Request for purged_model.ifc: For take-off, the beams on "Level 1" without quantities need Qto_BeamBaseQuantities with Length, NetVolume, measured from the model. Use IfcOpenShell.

First a look at what the model holds.

```python
import ifcopenshell
import ifcopenshell.util.element
import ifcopenshell.util.unit

model = ifcopenshell.open("purged_model.ifc")
print(model.schema)
for unit_type in ("LENGTHUNIT", "AREAUNIT", "VOLUMEUNIT"):
    print(unit_type, ifcopenshell.util.unit.calculate_unit_scale(model, unit_type))
storey = next(s for s in model.by_type("IfcBuildingStorey") if s.Name == "Level 1")
beams = [e for e in ifcopenshell.util.element.get_decomposition(storey) if e.is_a("IfcBeam")]
for e in sorted(beams, key=lambda e: e.id()):
    print(e.id(), e.is_a(), e.Name, list(ifcopenshell.util.element.get_psets(e, qtos_only=True)), sep=" | ")
```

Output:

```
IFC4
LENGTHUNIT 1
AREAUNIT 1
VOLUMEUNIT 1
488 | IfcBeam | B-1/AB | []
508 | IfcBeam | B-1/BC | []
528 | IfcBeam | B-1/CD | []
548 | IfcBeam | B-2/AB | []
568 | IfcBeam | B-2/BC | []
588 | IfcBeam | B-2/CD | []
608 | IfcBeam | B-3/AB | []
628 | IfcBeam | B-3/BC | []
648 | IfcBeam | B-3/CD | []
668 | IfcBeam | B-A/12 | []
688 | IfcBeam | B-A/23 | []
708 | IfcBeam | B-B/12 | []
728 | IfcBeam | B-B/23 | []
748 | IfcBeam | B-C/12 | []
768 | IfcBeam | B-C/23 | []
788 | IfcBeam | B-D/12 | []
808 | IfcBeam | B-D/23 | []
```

```python
import ifcopenshell
import ifcopenshell.api.pset
import ifcopenshell.geom
import ifcopenshell.util.element
import ifcopenshell.util.shape
import ifcopenshell.util.unit

model = ifcopenshell.open("purged_model.ifc")
unit_scale = ifcopenshell.util.unit.calculate_unit_scale(model)
volume_scale = ifcopenshell.util.unit.calculate_unit_scale(model, "VOLUMEUNIT")
settings = ifcopenshell.geom.settings()

storey = next(s for s in model.by_type("IfcBuildingStorey") if s.Name == "Level 1")
beams = [e for e in ifcopenshell.util.element.get_decomposition(storey) if e.is_a("IfcBeam")]

for e in sorted(beams, key=lambda e: e.id()):
    if ifcopenshell.util.element.get_psets(e, qtos_only=True, should_inherit=False):
        continue
    # Geometry comes back in metres, in the element's own axes.
    shape = ifcopenshell.geom.create_shape(settings, e)
    values = {
        "Length": ifcopenshell.util.shape.get_max_xyz(shape.geometry) / unit_scale,
        "NetVolume": ifcopenshell.util.shape.get_volume(shape.geometry) / volume_scale,
    }
    qto = ifcopenshell.api.pset.add_qto(model, product=e, name="Qto_BeamBaseQuantities")
    ifcopenshell.api.pset.edit_qto(model, qto=qto, properties=values)
    print(e.id(), {k: round(v, 3) for k, v in values.items()})

model.write("purged_model_rev.ifc")
```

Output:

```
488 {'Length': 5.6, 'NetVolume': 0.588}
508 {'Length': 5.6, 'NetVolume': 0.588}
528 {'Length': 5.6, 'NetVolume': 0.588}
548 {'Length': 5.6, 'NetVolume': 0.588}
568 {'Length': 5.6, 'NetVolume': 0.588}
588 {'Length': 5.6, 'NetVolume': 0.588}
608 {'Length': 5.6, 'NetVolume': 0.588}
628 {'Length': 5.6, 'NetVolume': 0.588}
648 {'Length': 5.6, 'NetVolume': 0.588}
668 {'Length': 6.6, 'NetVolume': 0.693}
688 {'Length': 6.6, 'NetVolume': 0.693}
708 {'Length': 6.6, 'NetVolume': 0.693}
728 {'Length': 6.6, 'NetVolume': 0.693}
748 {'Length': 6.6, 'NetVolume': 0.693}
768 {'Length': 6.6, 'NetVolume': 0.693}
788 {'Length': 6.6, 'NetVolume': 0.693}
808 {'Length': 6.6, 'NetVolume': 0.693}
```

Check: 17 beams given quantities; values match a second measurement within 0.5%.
